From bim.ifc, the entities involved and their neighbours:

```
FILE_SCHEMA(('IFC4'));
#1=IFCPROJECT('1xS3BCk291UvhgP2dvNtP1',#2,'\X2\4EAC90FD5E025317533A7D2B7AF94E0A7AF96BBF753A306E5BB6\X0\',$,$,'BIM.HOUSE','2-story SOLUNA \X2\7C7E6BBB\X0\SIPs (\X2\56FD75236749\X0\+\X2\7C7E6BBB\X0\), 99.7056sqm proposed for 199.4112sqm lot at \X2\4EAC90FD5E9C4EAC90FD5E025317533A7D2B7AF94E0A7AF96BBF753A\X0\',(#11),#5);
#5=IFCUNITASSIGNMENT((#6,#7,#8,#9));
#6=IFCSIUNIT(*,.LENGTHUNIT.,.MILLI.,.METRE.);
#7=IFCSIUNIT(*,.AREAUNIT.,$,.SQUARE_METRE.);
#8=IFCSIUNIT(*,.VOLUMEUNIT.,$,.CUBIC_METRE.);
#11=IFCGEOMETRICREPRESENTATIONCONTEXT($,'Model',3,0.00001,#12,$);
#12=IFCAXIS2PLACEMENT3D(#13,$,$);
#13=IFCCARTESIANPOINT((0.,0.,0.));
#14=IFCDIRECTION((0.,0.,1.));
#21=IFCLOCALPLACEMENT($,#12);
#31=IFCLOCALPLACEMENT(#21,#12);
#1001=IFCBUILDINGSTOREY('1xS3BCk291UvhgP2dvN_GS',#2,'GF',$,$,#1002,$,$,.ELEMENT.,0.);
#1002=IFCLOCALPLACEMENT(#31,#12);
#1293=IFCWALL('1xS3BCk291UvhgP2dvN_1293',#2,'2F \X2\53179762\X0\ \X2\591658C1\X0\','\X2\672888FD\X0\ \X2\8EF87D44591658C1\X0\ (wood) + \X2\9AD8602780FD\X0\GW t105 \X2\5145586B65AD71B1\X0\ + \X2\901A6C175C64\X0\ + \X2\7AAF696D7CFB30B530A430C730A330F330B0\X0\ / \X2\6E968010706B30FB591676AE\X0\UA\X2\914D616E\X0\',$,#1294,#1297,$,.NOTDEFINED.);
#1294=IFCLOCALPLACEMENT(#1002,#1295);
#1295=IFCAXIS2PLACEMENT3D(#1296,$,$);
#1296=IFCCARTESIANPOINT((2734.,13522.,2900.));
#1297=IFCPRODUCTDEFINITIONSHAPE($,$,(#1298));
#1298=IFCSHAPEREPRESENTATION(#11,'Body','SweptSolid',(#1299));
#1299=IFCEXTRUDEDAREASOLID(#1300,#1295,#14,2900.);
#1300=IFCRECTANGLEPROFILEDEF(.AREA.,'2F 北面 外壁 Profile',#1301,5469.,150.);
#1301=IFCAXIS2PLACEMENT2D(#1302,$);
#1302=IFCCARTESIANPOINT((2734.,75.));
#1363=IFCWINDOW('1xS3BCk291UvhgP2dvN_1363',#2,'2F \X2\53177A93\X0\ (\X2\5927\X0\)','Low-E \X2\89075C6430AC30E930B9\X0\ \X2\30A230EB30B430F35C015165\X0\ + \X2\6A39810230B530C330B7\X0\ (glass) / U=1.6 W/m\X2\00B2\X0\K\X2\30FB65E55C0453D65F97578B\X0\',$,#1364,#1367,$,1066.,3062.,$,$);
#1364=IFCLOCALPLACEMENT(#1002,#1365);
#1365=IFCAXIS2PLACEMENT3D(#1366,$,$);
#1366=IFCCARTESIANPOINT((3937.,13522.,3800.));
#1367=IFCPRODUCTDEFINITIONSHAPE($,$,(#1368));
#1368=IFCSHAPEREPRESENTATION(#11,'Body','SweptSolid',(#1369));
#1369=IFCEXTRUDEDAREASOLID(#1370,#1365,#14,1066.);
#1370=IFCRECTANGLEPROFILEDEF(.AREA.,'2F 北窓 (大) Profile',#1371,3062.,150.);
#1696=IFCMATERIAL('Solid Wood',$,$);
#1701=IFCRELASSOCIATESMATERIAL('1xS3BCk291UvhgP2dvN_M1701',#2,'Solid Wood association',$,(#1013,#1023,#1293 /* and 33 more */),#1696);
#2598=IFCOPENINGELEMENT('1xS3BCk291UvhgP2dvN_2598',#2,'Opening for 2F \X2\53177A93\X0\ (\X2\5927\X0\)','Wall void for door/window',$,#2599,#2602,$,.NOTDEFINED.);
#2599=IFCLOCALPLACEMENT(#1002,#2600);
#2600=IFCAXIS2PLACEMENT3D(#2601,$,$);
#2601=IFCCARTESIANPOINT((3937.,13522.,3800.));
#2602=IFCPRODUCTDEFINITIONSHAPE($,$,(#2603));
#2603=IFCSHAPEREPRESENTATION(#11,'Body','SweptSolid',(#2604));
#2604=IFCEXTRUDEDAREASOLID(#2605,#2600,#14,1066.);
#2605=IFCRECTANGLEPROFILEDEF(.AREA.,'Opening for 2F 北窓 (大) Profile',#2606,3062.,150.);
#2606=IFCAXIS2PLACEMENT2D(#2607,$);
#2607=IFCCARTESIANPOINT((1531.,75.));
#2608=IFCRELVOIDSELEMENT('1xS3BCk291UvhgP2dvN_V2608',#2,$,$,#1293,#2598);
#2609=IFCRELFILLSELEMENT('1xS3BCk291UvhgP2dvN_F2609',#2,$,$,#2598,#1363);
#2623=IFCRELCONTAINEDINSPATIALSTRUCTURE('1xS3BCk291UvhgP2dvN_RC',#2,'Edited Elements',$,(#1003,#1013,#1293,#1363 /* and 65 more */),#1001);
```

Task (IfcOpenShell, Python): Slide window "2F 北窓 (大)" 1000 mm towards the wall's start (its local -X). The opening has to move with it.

```python
import ifcopenshell
import ifcopenshell.api.geometry
import ifcopenshell.util.placement
import ifcopenshell.util.unit

model = ifcopenshell.open("bim.ifc")
unit_scale = ifcopenshell.util.unit.calculate_unit_scale(model)

window = model.by_id(1363)
opening = window.FillsVoids[0].RelatingOpeningElement
wall = opening.VoidsElements[0].RelatingBuildingElement

wall_matrix = ifcopenshell.util.placement.get_local_placement(wall.ObjectPlacement)
shift = wall_matrix[:3, 0] * -1 / unit_scale
before = ifcopenshell.util.placement.get_local_placement(window.ObjectPlacement)[:3, 3].copy()

# The window is not placed relative to its opening, so move both.
for product in (opening, window):
    matrix = ifcopenshell.util.placement.get_local_placement(product.ObjectPlacement)
    matrix[:3, 3] += shift
    ifcopenshell.api.geometry.edit_object_placement(model, product=product, matrix=matrix, is_si=False)

after = ifcopenshell.util.placement.get_local_placement(window.ObjectPlacement)[:3, 3]
print("window moved by", (after - before).round(3) + 0.0)

model.write("bim_v2.ifc")
```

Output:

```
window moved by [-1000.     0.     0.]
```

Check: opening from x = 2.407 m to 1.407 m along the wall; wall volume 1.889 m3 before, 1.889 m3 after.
